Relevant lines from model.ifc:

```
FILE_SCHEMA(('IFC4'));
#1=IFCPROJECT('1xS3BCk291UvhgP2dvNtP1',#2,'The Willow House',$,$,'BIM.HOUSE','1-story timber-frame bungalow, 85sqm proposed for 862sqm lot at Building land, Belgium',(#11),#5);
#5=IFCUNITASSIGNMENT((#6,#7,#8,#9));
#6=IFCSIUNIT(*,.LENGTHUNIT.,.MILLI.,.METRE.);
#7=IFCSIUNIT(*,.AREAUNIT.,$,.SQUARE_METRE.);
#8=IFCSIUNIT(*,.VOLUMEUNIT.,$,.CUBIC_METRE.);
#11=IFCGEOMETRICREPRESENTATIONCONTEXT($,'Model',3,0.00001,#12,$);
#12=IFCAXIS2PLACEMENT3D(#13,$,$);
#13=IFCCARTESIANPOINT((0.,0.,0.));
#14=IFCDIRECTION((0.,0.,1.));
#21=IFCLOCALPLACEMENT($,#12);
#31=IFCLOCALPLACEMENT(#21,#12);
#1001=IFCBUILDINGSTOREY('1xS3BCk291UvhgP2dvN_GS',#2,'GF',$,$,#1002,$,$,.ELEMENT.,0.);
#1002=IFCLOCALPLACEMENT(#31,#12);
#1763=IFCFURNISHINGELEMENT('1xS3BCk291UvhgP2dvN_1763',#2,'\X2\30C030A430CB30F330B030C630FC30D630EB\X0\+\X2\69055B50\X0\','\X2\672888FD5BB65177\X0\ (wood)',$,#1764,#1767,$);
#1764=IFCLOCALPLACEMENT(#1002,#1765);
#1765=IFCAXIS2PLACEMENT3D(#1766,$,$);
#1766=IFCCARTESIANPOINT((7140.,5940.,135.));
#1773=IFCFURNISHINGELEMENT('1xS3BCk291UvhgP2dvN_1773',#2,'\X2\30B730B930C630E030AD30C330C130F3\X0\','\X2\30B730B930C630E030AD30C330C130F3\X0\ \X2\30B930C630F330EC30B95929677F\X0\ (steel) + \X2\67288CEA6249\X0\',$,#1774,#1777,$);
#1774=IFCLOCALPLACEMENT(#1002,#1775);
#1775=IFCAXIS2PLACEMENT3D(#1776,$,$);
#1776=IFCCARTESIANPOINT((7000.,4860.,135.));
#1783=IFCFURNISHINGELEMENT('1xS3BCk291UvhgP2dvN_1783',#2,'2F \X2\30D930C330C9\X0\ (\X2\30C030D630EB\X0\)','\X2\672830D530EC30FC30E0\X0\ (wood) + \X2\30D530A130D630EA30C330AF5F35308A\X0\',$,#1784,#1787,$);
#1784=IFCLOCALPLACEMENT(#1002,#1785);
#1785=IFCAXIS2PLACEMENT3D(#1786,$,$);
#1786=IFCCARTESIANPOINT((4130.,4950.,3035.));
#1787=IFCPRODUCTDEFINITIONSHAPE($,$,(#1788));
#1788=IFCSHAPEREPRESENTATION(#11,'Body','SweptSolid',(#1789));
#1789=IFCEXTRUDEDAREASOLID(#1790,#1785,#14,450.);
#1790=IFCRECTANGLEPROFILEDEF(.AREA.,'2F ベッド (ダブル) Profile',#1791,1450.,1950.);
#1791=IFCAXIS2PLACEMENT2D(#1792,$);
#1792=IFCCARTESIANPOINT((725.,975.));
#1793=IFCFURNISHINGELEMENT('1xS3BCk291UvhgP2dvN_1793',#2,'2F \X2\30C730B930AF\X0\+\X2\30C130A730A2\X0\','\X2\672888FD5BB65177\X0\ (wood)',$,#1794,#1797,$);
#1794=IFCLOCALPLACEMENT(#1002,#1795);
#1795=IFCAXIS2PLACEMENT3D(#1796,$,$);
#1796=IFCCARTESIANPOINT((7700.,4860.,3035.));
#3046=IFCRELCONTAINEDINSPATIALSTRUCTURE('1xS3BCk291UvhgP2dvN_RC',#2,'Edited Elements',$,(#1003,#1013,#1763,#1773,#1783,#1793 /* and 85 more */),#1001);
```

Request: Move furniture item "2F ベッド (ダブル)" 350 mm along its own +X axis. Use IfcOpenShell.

```python
import ifcopenshell
import ifcopenshell.api.geometry
import ifcopenshell.util.placement
import ifcopenshell.util.unit

model = ifcopenshell.open("model.ifc")
unit_scale = ifcopenshell.util.unit.calculate_unit_scale(model)

item = model.by_guid("1xS3BCk291UvhgP2dvN_1783")
matrix = ifcopenshell.util.placement.get_local_placement(item.ObjectPlacement)
matrix[:3, 3] += matrix[:3, 0] * 0.35 / unit_scale
ifcopenshell.api.geometry.edit_object_placement(model, product=item, matrix=matrix, is_si=False)

print(ifcopenshell.util.placement.get_local_placement(item.ObjectPlacement).round(3) + 0.0)

model.write("model_updated.ifc")
```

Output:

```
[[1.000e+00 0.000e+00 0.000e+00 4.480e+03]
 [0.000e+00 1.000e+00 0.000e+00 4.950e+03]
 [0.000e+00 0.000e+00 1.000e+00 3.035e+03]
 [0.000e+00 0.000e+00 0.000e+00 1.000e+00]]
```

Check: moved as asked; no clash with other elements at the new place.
